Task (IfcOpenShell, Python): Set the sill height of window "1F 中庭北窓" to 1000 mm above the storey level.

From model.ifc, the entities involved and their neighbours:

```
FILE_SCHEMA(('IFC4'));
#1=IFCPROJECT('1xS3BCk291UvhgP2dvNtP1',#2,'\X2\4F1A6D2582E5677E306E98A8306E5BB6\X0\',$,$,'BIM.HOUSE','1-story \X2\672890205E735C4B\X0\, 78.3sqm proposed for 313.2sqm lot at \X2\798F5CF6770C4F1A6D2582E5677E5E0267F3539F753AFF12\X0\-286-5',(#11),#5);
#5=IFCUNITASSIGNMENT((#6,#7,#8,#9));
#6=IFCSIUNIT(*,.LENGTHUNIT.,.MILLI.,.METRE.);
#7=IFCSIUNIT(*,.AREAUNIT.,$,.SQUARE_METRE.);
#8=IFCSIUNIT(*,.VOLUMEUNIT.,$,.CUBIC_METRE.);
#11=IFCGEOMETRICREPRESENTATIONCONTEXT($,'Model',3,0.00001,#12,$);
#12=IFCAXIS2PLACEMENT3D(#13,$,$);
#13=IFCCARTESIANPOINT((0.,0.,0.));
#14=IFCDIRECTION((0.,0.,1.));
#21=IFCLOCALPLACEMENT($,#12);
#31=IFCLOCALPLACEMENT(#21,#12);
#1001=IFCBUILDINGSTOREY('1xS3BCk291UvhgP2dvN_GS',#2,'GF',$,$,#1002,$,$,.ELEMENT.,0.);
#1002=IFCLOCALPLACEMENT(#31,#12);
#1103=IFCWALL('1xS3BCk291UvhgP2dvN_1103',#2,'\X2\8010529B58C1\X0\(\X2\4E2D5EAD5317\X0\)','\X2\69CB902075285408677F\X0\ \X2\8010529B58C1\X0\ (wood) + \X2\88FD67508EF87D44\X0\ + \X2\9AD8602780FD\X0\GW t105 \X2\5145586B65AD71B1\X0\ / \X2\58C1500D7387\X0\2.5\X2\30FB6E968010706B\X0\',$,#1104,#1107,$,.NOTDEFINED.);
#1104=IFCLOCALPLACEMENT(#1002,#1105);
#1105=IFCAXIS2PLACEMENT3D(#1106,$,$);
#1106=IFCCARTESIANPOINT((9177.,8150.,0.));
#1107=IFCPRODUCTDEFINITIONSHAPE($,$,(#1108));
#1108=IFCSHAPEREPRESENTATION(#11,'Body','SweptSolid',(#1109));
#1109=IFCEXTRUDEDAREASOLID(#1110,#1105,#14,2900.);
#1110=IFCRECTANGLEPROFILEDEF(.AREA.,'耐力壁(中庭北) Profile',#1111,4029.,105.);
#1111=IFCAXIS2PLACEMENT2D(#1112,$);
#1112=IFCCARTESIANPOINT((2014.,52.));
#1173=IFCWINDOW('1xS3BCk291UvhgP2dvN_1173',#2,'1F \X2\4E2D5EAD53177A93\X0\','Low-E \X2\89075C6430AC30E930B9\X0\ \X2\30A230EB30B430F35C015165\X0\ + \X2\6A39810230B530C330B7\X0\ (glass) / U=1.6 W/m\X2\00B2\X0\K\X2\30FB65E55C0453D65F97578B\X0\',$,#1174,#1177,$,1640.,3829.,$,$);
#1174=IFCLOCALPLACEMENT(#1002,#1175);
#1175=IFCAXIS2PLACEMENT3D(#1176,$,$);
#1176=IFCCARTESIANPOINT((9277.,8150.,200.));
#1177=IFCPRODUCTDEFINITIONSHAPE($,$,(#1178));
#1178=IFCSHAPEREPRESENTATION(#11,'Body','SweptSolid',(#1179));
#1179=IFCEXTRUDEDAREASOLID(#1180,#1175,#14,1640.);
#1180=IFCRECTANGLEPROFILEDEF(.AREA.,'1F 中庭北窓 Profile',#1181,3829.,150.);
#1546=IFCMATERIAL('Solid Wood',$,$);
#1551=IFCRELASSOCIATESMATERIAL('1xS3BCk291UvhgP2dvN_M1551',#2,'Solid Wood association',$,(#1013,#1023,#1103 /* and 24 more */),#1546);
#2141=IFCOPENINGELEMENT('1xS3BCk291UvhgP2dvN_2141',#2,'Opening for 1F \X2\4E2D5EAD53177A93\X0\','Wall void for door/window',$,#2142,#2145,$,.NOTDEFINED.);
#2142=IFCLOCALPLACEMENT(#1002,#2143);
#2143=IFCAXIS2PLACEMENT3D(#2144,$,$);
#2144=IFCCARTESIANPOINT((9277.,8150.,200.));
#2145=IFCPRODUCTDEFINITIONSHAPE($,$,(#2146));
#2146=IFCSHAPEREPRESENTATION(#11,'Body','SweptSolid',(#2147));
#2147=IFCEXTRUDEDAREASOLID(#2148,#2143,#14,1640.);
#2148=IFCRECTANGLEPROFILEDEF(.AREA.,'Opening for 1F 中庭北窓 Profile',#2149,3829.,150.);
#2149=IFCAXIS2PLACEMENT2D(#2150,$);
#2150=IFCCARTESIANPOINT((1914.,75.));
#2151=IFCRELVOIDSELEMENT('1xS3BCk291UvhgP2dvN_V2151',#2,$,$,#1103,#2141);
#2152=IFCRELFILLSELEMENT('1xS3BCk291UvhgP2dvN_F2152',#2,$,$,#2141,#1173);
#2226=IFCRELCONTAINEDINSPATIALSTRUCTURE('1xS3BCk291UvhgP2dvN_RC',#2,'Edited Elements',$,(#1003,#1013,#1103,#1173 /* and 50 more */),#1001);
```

```python
import numpy as np
import ifcopenshell
import ifcopenshell.api.geometry
import ifcopenshell.geom
import ifcopenshell.util.element
import ifcopenshell.util.placement
import ifcopenshell.util.shape
import ifcopenshell.util.unit

model = ifcopenshell.open("model.ifc")
unit_scale = ifcopenshell.util.unit.calculate_unit_scale(model)

window = model.by_id(1173)
opening = window.FillsVoids[0].RelatingOpeningElement
storey = ifcopenshell.util.element.get_container(window, ifc_class="IfcBuildingStorey")
level = ifcopenshell.util.placement.get_local_placement(storey.ObjectPlacement)[2, 3]

# The opening's origin need not be at the sill, so measure its lowest point.
shape = ifcopenshell.geom.create_shape(ifcopenshell.geom.settings(), opening)
bottom = ifcopenshell.util.shape.get_shape_bottom_elevation(shape, shape.geometry) / unit_scale
dz = level + 1000.0 - bottom

shift = np.array([0.0, 0.0, dz])
# The window is not placed relative to its opening, so move both.
for product in (opening, window):
    matrix = ifcopenshell.util.placement.get_local_placement(product.ObjectPlacement)
    matrix[:3, 3] += shift
    ifcopenshell.api.geometry.edit_object_placement(model, product=product, matrix=matrix, is_si=False)

print(f"moved by {dz * unit_scale:+.3f} m")

model.write("model_edited.ifc")
```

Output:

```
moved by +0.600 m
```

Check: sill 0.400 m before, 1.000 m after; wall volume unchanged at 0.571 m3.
